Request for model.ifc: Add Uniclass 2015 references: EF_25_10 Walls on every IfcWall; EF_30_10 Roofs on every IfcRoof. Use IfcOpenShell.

First a look at what the model holds.

```python
import ifcopenshell

model = ifcopenshell.open("model.ifc")
print(model.schema)
print("classifications:", [c.Name for c in model.by_type("IfcClassification")])
for ifc_class in ("IfcDoor", "IfcRoof", "IfcStair", "IfcWall", "IfcWindow"):
    print(ifc_class, len(model.by_type(ifc_class)))
```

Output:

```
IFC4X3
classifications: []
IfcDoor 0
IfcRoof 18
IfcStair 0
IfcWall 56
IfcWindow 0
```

```python
import ifcopenshell
import ifcopenshell.api.classification

model = ifcopenshell.open("model.ifc")

system = ifcopenshell.api.classification.add_classification(model, classification="Uniclass 2015")

codes = {
    "IfcWall": ("EF_25_10", "Walls"),
    "IfcRoof": ("EF_30_10", "Roofs"),
}
for ifc_class, (code, name) in codes.items():
    products = model.by_type(ifc_class)
    ifcopenshell.api.classification.add_reference(
        model, products=products, classification=system, identification=code, name=name
    )
    print(code, len(products))

model.write("model_updated.ifc")
```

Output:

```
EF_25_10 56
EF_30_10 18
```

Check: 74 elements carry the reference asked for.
